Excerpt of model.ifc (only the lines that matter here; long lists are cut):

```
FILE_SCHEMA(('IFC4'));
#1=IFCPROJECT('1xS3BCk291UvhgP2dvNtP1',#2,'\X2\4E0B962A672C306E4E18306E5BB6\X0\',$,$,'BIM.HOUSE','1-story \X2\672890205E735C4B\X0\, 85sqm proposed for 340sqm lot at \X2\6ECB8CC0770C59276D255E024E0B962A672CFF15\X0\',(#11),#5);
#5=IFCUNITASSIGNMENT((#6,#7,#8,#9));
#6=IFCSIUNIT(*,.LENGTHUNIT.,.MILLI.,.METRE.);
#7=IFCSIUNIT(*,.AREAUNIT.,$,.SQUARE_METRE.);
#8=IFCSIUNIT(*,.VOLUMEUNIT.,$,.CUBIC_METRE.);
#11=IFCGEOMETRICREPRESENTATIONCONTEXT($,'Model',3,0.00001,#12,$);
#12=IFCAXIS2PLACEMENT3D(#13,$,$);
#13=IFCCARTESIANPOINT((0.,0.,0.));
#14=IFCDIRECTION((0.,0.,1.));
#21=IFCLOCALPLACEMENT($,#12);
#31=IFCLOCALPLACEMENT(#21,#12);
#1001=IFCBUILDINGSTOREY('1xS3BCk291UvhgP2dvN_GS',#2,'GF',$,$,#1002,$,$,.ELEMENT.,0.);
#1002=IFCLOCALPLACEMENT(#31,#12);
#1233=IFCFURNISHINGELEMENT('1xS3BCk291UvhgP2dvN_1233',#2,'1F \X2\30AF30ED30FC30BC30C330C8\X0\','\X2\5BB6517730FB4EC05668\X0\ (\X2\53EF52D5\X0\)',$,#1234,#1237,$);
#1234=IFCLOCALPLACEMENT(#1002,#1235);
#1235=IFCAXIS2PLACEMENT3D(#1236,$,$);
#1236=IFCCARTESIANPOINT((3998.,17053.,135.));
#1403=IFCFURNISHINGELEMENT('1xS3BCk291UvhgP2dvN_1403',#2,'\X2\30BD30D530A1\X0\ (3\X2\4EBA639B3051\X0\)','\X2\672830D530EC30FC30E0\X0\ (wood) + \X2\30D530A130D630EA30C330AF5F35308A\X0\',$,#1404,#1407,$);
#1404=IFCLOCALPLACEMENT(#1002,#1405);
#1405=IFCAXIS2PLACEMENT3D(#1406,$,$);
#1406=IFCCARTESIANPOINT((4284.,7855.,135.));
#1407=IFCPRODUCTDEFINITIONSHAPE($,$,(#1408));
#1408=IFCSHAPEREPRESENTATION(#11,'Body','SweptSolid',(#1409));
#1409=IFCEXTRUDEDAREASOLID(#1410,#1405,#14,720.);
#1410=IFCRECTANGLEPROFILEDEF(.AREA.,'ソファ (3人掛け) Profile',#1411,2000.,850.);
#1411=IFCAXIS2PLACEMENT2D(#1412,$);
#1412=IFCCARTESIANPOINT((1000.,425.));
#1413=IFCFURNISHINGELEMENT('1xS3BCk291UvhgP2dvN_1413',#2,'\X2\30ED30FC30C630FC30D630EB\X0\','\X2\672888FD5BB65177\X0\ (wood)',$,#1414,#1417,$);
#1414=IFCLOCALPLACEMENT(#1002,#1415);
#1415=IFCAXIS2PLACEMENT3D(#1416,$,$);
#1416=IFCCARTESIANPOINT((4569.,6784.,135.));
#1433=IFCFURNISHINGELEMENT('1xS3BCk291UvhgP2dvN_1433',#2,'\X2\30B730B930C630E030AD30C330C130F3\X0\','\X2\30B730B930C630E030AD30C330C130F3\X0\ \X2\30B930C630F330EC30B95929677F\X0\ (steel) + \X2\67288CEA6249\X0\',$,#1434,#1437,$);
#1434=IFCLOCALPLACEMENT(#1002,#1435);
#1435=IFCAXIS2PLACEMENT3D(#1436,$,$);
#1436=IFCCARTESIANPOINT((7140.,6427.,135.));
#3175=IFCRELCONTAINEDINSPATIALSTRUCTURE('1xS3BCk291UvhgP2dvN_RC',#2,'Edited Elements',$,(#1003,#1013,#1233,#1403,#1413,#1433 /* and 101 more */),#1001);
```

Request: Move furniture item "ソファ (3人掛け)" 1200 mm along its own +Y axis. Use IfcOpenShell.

```python
import ifcopenshell
import ifcopenshell.api.geometry
import ifcopenshell.util.placement
import ifcopenshell.util.unit

model = ifcopenshell.open("model.ifc")
unit_scale = ifcopenshell.util.unit.calculate_unit_scale(model)

item = model.by_guid("1xS3BCk291UvhgP2dvN_1403")
matrix = ifcopenshell.util.placement.get_local_placement(item.ObjectPlacement)
matrix[:3, 3] += matrix[:3, 1] * 1.2 / unit_scale
ifcopenshell.api.geometry.edit_object_placement(model, product=item, matrix=matrix, is_si=False)

print(ifcopenshell.util.placement.get_local_placement(item.ObjectPlacement).round(3) + 0.0)

model.write("model_rev.ifc")
```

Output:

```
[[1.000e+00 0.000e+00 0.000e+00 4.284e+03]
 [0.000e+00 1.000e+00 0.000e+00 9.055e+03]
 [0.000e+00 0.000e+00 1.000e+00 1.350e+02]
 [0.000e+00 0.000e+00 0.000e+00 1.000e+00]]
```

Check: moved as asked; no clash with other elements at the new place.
